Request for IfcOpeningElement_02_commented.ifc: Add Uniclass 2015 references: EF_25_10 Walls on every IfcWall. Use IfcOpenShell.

First a look at what the model holds.

```python
import ifcopenshell

model = ifcopenshell.open("IfcOpeningElement_02_commented.ifc")
print(model.schema)
print("classifications:", [c.Name for c in model.by_type("IfcClassification")])
for ifc_class in ("IfcDoor", "IfcRoof", "IfcStair", "IfcWall", "IfcWindow"):
    print(ifc_class, len(model.by_type(ifc_class)))
```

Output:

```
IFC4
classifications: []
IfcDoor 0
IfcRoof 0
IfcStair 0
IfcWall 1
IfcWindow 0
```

```python
import ifcopenshell
import ifcopenshell.api.classification

model = ifcopenshell.open("IfcOpeningElement_02_commented.ifc")

system = ifcopenshell.api.classification.add_classification(model, classification="Uniclass 2015")

codes = {
    "IfcWall": ("EF_25_10", "Walls"),
}
for ifc_class, (code, name) in codes.items():
    products = model.by_type(ifc_class)
    ifcopenshell.api.classification.add_reference(
        model, products=products, classification=system, identification=code, name=name
    )
    print(code, len(products))

model.write("IfcOpeningElement_02_commented_v2.ifc")
```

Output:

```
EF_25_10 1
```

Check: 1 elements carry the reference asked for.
